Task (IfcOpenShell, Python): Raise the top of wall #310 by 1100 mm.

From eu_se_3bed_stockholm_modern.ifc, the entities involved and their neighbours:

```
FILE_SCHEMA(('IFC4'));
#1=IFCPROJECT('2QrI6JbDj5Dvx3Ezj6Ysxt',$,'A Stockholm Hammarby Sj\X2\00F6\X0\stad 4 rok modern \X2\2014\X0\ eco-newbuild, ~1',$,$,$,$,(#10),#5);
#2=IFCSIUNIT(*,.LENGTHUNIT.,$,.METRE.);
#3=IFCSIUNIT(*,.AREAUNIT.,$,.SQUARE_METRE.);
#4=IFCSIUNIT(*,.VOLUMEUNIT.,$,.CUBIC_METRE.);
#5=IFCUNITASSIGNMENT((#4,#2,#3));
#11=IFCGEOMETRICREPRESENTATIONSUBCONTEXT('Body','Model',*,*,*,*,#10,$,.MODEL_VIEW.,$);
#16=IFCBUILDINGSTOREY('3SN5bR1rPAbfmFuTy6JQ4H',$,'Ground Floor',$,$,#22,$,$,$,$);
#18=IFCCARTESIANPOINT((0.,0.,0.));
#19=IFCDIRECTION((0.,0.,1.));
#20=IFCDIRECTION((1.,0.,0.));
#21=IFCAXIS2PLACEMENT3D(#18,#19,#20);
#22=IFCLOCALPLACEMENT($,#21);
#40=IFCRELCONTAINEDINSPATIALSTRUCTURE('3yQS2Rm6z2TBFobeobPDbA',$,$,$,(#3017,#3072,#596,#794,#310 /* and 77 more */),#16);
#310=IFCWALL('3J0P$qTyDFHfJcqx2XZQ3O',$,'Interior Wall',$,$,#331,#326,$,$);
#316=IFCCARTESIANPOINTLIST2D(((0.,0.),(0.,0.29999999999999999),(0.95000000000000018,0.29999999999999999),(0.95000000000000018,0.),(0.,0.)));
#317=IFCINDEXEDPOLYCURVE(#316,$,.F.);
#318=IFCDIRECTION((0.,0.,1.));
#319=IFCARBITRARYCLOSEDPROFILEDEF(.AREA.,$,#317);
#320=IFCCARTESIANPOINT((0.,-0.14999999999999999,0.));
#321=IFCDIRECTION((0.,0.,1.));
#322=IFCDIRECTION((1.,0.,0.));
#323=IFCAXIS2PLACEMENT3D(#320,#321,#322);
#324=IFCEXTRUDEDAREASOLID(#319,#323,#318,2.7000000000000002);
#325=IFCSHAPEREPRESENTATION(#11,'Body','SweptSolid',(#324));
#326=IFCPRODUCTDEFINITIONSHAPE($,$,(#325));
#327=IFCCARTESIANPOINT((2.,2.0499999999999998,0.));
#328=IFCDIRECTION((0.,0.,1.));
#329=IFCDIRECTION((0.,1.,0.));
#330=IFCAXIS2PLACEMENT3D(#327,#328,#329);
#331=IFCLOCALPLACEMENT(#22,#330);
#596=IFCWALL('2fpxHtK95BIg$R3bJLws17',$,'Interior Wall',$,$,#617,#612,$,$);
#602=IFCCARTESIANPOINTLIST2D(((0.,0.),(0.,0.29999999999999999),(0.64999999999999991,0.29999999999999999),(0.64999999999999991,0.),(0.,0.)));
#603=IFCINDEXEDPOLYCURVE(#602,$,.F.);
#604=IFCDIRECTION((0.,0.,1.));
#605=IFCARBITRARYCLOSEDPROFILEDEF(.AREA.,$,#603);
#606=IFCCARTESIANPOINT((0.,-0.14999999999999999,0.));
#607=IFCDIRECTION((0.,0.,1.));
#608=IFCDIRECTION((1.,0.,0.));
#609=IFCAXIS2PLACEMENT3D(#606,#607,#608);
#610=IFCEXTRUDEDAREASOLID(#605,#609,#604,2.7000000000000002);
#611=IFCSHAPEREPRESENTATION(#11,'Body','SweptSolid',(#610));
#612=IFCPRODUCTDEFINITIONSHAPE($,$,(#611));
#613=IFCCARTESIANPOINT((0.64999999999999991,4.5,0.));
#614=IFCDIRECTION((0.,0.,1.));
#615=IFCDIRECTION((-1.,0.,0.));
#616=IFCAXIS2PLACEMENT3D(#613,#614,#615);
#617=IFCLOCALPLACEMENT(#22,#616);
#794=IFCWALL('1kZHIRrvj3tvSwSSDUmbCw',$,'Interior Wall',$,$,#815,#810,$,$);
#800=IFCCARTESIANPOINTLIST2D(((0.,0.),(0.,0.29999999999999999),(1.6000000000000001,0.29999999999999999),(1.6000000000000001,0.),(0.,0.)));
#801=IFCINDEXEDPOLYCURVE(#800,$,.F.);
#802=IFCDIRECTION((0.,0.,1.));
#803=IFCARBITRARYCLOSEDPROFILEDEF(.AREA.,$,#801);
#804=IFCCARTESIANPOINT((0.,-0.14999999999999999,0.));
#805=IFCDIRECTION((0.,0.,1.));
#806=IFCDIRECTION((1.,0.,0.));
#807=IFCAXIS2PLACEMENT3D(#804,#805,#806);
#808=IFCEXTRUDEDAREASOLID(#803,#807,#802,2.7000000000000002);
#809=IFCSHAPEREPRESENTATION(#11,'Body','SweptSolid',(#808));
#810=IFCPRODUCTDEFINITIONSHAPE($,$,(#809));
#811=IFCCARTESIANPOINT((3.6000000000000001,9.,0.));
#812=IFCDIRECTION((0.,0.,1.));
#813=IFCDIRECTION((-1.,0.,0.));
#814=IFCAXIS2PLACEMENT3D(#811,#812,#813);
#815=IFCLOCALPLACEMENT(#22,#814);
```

```python
import ifcopenshell
import ifcopenshell.geom
import ifcopenshell.util.representation
import ifcopenshell.util.shape
import ifcopenshell.util.unit

model = ifcopenshell.open("eu_se_3bed_stockholm_modern.ifc")
unit_scale = ifcopenshell.util.unit.calculate_unit_scale(model)
settings = ifcopenshell.geom.settings()


def volume(element):
    """Net volume in cubic metres, openings subtracted."""
    shape = ifcopenshell.geom.create_shape(settings, element)
    return ifcopenshell.util.shape.get_volume(shape.geometry)


wall = model.by_guid("3J0P$qTyDFHfJcqx2XZQ3O")
before = volume(wall)

body = ifcopenshell.util.representation.get_representation(wall, "Model", "Body")
solid = body.Items[0]
old_height = solid.Depth
solid.Depth += 1.1 / unit_scale
after = volume(wall)

print(f"height {old_height:g} -> {solid.Depth:g}, volume {before:.3f} -> {after:.3f} m3")

model.write("eu_se_3bed_stockholm_modern_edited.ifc")
```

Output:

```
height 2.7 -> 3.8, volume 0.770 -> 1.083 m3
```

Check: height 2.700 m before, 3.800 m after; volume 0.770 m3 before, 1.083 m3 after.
